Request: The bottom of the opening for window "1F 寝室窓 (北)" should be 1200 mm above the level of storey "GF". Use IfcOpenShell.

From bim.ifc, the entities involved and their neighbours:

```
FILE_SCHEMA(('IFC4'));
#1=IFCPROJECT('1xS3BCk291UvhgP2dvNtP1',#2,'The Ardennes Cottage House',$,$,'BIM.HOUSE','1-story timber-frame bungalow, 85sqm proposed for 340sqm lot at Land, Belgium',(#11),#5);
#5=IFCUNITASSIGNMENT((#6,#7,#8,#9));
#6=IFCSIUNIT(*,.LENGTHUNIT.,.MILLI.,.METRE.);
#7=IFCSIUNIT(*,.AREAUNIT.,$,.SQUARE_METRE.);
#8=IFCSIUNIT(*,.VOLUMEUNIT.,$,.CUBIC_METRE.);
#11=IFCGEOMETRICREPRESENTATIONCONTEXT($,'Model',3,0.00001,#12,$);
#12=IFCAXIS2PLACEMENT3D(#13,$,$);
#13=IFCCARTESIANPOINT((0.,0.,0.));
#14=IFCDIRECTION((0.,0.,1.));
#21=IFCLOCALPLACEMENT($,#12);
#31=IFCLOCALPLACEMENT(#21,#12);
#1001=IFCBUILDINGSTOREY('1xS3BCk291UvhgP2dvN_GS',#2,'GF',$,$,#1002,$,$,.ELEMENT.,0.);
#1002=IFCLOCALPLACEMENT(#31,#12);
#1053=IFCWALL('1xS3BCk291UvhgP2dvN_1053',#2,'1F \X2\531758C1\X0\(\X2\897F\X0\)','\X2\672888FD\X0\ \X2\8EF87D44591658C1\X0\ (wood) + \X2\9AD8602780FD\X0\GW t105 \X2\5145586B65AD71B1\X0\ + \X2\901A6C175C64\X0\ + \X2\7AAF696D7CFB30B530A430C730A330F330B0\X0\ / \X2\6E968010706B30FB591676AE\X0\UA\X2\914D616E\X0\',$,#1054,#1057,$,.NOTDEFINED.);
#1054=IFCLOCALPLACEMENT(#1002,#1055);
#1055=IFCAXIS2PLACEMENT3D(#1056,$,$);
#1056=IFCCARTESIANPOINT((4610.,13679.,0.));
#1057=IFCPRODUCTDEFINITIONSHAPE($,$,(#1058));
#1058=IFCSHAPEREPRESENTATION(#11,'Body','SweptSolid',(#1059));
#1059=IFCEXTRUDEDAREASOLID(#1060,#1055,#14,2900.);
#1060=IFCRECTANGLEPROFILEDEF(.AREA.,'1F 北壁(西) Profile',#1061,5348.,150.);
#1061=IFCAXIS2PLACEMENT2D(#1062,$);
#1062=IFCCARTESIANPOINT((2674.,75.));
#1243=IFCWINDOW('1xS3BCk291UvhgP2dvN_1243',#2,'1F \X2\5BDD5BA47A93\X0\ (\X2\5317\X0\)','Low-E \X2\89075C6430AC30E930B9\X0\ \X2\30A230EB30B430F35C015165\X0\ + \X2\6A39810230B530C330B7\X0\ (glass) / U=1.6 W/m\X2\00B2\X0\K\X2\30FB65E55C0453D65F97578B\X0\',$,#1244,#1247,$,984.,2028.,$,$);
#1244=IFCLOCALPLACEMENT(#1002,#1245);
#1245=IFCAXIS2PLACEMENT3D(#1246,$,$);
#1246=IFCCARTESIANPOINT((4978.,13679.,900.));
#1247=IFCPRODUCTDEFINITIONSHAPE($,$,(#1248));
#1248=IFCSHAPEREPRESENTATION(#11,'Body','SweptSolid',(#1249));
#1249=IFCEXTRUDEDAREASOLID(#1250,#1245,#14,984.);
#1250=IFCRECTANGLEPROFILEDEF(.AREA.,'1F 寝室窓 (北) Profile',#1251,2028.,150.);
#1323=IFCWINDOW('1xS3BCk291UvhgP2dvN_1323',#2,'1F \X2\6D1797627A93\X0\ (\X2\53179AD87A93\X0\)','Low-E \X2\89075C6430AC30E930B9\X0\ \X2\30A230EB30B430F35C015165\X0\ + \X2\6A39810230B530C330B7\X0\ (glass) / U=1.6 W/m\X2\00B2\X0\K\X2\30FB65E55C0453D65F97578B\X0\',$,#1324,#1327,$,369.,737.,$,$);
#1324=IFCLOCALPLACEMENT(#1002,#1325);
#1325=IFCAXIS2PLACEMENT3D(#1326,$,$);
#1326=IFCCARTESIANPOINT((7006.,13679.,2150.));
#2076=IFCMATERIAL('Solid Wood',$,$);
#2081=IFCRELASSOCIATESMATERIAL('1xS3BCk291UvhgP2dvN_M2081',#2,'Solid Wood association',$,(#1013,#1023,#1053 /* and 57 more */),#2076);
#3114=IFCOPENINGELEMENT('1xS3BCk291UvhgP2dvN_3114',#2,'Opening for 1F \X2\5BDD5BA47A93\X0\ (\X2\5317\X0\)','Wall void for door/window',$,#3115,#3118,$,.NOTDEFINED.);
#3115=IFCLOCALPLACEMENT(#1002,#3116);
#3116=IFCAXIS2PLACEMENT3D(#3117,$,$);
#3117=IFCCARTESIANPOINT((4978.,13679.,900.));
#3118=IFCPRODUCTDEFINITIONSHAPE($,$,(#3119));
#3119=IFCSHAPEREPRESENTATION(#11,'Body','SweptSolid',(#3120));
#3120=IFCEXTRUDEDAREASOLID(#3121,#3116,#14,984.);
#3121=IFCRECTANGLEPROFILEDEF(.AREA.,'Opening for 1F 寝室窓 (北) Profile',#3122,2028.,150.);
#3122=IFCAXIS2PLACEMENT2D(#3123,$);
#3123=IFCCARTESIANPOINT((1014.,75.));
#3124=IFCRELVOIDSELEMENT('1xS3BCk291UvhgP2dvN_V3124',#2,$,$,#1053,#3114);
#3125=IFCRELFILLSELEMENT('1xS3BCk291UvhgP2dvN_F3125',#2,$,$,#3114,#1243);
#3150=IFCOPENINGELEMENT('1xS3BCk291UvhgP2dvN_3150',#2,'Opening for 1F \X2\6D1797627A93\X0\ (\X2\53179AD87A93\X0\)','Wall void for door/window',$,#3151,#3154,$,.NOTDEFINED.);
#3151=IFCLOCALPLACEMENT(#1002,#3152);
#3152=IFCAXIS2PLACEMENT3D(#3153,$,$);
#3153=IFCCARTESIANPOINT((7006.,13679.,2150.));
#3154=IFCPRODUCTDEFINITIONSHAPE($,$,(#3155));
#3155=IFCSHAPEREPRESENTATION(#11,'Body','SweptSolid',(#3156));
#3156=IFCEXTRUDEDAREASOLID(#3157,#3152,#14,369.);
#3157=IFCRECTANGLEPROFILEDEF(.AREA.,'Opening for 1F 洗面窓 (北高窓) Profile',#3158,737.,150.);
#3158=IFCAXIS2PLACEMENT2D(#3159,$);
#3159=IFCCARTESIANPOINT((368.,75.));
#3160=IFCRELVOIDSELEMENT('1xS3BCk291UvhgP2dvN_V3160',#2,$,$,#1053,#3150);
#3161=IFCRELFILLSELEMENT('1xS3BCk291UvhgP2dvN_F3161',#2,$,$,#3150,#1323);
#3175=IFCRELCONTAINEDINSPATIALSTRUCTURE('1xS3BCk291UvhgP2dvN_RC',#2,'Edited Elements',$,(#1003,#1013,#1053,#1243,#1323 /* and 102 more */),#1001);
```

```python
import numpy as np
import ifcopenshell
import ifcopenshell.api.geometry
import ifcopenshell.geom
import ifcopenshell.util.element
import ifcopenshell.util.placement
import ifcopenshell.util.shape
import ifcopenshell.util.unit

model = ifcopenshell.open("bim.ifc")
unit_scale = ifcopenshell.util.unit.calculate_unit_scale(model)

window = model.by_guid("1xS3BCk291UvhgP2dvN_1243")
opening = window.FillsVoids[0].RelatingOpeningElement
storey = ifcopenshell.util.element.get_container(window, ifc_class="IfcBuildingStorey")
level = ifcopenshell.util.placement.get_local_placement(storey.ObjectPlacement)[2, 3]

# The opening's origin need not be at the sill, so measure its lowest point.
shape = ifcopenshell.geom.create_shape(ifcopenshell.geom.settings(), opening)
bottom = ifcopenshell.util.shape.get_shape_bottom_elevation(shape, shape.geometry) / unit_scale
dz = level + 1.2 / unit_scale - bottom

shift = np.array([0.0, 0.0, dz])
# The window is not placed relative to its opening, so move both.
for product in (opening, window):
    matrix = ifcopenshell.util.placement.get_local_placement(product.ObjectPlacement)
    matrix[:3, 3] += shift
    ifcopenshell.api.geometry.edit_object_placement(model, product=product, matrix=matrix, is_si=False)

print(f"moved by {dz * unit_scale:+.3f} m")

model.write("bim-out.ifc")
```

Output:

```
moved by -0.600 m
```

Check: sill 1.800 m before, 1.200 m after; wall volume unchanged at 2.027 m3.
